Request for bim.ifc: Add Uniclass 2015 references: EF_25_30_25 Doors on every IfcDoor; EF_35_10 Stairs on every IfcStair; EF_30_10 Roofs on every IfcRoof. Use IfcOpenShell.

First a look at what the model holds.

```python
import ifcopenshell

model = ifcopenshell.open("bim.ifc")
print(model.schema)
print("classifications:", [c.Name for c in model.by_type("IfcClassification")])
for ifc_class in ("IfcDoor", "IfcRoof", "IfcStair", "IfcWall", "IfcWindow"):
    print(ifc_class, len(model.by_type(ifc_class)))
```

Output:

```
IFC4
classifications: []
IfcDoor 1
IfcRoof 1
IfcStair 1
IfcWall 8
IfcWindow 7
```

```python
import ifcopenshell
import ifcopenshell.api.classification

model = ifcopenshell.open("bim.ifc")

system = ifcopenshell.api.classification.add_classification(model, classification="Uniclass 2015")

codes = {
    "IfcDoor": ("EF_25_30_25", "Doors"),
    "IfcStair": ("EF_35_10", "Stairs"),
    "IfcRoof": ("EF_30_10", "Roofs"),
}
for ifc_class, (code, name) in codes.items():
    products = model.by_type(ifc_class)
    ifcopenshell.api.classification.add_reference(
        model, products=products, classification=system, identification=code, name=name
    )
    print(code, len(products))

model.write("bim_rev.ifc")
```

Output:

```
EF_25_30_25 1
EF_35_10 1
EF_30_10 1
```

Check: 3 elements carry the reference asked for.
